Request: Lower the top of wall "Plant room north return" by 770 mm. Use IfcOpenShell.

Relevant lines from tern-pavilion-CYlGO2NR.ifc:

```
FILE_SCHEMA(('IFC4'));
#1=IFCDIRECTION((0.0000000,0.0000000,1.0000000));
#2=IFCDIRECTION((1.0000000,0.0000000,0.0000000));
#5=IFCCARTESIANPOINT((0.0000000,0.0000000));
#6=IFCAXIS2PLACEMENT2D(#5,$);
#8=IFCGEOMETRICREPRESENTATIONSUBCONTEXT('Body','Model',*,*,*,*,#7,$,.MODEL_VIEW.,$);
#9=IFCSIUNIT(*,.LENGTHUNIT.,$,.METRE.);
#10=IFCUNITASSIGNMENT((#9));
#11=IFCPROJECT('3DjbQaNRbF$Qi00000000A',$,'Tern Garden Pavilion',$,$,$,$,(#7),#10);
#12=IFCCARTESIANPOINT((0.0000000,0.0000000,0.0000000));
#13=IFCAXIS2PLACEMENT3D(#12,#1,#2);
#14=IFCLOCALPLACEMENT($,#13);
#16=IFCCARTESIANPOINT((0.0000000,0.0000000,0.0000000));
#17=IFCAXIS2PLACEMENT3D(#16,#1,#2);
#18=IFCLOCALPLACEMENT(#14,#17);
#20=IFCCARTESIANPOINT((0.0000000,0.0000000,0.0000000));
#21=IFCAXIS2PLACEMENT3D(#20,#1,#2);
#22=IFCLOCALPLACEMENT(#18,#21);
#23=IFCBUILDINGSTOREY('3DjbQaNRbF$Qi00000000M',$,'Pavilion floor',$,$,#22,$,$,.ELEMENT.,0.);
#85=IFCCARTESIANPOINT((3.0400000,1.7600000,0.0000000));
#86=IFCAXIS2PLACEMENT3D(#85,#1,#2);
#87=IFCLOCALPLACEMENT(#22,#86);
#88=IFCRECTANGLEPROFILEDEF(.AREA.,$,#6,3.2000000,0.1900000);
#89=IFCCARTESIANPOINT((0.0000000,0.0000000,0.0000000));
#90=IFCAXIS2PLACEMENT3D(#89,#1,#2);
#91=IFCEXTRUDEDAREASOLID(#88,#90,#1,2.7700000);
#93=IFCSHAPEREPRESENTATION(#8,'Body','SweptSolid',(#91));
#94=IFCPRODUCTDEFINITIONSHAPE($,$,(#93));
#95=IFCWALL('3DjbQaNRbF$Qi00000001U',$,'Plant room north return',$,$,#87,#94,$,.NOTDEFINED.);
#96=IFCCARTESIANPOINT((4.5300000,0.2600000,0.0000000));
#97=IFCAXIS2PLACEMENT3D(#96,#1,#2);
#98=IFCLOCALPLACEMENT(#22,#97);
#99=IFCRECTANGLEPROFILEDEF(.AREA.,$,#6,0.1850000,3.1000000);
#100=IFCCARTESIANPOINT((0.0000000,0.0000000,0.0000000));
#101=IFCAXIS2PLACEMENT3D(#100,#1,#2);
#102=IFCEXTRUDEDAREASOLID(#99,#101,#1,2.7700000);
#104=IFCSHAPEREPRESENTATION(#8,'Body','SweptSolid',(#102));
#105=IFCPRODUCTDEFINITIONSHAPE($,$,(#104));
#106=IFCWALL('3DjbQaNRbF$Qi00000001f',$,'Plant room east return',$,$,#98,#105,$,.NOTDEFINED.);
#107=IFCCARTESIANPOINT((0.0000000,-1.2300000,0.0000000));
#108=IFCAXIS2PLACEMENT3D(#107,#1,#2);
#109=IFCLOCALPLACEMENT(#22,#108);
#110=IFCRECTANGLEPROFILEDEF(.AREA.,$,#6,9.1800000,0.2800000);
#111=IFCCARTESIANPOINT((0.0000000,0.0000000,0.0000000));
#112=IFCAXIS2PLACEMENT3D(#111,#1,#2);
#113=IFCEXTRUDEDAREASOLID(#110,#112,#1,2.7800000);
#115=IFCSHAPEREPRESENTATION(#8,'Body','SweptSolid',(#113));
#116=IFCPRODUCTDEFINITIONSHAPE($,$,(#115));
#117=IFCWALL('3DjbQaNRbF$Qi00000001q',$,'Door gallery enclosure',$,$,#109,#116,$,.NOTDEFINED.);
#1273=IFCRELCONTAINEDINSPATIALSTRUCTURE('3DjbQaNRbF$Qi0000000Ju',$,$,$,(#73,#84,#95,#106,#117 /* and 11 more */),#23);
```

```python
import ifcopenshell
import ifcopenshell.geom
import ifcopenshell.util.representation
import ifcopenshell.util.shape

model = ifcopenshell.open("tern-pavilion-CYlGO2NR.ifc")
settings = ifcopenshell.geom.settings()


def volume(element):
    """Net volume in cubic metres, openings subtracted."""
    shape = ifcopenshell.geom.create_shape(settings, element)
    return ifcopenshell.util.shape.get_volume(shape.geometry)


wall = model.by_id(95)
before = volume(wall)

body = ifcopenshell.util.representation.get_representation(wall, "Model", "Body")
solid = body.Items[0]
old_height = solid.Depth
solid.Depth -= 0.77
after = volume(wall)

print(f"height {old_height:g} -> {solid.Depth:g}, volume {before:.3f} -> {after:.3f} m3")

model.write("tern-pavilion-CYlGO2NR-out.ifc")
```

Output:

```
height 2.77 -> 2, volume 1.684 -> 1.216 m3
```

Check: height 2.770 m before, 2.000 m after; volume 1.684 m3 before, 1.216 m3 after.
